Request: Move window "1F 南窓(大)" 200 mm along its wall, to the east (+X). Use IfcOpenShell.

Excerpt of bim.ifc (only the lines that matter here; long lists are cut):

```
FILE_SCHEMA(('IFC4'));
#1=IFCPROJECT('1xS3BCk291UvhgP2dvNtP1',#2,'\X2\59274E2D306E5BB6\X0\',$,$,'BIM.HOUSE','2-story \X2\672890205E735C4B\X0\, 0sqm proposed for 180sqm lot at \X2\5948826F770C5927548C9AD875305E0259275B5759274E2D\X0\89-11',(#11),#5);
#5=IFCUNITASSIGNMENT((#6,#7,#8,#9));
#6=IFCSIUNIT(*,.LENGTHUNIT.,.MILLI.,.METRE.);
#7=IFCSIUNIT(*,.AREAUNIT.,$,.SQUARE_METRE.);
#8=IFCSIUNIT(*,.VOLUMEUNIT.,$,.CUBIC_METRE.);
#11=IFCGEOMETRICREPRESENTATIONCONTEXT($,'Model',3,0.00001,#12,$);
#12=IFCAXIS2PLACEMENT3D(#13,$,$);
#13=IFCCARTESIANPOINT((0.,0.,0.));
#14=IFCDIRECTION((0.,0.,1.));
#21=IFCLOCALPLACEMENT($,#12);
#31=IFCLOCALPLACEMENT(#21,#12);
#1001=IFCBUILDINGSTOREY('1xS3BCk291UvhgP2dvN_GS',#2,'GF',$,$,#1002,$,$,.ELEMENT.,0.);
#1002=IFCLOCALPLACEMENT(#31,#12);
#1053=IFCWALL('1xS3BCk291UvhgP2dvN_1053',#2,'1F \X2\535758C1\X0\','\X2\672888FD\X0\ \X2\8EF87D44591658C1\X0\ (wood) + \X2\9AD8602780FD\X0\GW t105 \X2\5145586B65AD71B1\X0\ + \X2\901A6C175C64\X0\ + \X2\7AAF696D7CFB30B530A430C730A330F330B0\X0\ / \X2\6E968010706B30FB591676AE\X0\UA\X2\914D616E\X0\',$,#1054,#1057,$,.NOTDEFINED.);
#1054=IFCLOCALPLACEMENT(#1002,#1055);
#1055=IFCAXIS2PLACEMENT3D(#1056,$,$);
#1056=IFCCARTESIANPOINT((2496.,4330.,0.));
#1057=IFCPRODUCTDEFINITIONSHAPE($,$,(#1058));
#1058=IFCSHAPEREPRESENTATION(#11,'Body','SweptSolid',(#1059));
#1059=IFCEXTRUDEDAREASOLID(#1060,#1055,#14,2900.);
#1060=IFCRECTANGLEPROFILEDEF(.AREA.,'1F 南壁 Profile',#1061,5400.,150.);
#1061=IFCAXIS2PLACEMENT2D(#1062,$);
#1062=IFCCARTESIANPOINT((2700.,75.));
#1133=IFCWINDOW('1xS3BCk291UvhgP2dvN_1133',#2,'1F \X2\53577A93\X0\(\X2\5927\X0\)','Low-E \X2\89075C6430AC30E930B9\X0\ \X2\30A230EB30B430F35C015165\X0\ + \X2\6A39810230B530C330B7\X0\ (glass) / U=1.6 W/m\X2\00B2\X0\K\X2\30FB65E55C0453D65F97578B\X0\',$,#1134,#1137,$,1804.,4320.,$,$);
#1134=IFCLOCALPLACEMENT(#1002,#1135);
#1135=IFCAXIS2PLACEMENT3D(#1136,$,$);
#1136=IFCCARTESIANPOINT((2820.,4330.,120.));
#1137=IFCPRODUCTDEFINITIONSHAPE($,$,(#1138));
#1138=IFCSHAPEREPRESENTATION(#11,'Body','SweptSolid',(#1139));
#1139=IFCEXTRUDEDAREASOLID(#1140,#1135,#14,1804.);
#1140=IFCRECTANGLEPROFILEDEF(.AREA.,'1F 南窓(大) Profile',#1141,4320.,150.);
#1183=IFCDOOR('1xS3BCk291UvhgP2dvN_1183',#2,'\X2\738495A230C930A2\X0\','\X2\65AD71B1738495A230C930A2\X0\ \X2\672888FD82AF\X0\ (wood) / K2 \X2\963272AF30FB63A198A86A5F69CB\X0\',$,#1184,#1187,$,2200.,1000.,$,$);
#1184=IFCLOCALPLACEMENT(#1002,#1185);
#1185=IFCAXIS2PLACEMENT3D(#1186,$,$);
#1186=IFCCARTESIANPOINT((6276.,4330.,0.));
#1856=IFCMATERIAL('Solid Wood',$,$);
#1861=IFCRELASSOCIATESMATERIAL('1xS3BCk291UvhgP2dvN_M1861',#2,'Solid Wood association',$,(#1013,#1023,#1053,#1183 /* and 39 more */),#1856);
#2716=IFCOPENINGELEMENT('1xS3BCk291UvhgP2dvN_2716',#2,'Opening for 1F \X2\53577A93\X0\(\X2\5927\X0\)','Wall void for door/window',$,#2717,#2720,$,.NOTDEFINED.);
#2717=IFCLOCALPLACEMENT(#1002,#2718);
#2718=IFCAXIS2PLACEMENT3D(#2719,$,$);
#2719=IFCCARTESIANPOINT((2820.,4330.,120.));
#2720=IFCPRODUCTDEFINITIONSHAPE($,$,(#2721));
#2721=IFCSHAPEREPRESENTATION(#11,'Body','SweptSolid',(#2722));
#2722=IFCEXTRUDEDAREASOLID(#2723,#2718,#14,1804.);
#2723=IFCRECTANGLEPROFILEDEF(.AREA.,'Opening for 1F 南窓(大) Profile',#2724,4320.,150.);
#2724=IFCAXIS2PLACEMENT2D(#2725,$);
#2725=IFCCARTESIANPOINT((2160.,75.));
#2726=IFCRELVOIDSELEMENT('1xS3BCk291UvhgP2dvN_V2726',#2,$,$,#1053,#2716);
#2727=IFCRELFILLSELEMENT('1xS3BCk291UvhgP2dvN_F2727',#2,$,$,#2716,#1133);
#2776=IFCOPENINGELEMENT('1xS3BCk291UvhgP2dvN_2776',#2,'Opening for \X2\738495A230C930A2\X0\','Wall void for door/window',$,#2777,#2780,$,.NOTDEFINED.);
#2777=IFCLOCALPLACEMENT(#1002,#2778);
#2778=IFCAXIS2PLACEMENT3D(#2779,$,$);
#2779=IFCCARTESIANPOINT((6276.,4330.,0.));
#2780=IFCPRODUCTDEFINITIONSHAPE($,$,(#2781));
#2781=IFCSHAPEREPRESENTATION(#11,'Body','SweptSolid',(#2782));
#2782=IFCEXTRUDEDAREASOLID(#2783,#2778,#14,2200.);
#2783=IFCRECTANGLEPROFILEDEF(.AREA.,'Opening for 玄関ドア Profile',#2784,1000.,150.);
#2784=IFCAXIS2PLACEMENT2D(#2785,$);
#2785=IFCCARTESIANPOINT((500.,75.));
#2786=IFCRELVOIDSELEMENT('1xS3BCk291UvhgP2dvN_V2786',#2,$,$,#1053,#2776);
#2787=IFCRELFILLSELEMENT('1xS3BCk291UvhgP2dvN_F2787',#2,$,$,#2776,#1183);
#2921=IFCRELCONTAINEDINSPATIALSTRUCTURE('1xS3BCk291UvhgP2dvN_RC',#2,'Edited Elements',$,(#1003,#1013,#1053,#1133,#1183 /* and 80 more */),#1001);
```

```python
import ifcopenshell
import ifcopenshell.api.geometry
import ifcopenshell.util.placement
import ifcopenshell.util.unit

model = ifcopenshell.open("bim.ifc")
unit_scale = ifcopenshell.util.unit.calculate_unit_scale(model)

window = model.by_guid("1xS3BCk291UvhgP2dvN_1133")
opening = window.FillsVoids[0].RelatingOpeningElement
wall = opening.VoidsElements[0].RelatingBuildingElement

wall_matrix = ifcopenshell.util.placement.get_local_placement(wall.ObjectPlacement)
shift = wall_matrix[:3, 0] * 0.2 / unit_scale
before = ifcopenshell.util.placement.get_local_placement(window.ObjectPlacement)[:3, 3].copy()

# The window is not placed relative to its opening, so move both.
for product in (opening, window):
    matrix = ifcopenshell.util.placement.get_local_placement(product.ObjectPlacement)
    matrix[:3, 3] += shift
    ifcopenshell.api.geometry.edit_object_placement(model, product=product, matrix=matrix, is_si=False)

after = ifcopenshell.util.placement.get_local_placement(window.ObjectPlacement)[:3, 3]
print("window moved by", (after - before).round(3) + 0.0)

model.write("bim_updated.ifc")
```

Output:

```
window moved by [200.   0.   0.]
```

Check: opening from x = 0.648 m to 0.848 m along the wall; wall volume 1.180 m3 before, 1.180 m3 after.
